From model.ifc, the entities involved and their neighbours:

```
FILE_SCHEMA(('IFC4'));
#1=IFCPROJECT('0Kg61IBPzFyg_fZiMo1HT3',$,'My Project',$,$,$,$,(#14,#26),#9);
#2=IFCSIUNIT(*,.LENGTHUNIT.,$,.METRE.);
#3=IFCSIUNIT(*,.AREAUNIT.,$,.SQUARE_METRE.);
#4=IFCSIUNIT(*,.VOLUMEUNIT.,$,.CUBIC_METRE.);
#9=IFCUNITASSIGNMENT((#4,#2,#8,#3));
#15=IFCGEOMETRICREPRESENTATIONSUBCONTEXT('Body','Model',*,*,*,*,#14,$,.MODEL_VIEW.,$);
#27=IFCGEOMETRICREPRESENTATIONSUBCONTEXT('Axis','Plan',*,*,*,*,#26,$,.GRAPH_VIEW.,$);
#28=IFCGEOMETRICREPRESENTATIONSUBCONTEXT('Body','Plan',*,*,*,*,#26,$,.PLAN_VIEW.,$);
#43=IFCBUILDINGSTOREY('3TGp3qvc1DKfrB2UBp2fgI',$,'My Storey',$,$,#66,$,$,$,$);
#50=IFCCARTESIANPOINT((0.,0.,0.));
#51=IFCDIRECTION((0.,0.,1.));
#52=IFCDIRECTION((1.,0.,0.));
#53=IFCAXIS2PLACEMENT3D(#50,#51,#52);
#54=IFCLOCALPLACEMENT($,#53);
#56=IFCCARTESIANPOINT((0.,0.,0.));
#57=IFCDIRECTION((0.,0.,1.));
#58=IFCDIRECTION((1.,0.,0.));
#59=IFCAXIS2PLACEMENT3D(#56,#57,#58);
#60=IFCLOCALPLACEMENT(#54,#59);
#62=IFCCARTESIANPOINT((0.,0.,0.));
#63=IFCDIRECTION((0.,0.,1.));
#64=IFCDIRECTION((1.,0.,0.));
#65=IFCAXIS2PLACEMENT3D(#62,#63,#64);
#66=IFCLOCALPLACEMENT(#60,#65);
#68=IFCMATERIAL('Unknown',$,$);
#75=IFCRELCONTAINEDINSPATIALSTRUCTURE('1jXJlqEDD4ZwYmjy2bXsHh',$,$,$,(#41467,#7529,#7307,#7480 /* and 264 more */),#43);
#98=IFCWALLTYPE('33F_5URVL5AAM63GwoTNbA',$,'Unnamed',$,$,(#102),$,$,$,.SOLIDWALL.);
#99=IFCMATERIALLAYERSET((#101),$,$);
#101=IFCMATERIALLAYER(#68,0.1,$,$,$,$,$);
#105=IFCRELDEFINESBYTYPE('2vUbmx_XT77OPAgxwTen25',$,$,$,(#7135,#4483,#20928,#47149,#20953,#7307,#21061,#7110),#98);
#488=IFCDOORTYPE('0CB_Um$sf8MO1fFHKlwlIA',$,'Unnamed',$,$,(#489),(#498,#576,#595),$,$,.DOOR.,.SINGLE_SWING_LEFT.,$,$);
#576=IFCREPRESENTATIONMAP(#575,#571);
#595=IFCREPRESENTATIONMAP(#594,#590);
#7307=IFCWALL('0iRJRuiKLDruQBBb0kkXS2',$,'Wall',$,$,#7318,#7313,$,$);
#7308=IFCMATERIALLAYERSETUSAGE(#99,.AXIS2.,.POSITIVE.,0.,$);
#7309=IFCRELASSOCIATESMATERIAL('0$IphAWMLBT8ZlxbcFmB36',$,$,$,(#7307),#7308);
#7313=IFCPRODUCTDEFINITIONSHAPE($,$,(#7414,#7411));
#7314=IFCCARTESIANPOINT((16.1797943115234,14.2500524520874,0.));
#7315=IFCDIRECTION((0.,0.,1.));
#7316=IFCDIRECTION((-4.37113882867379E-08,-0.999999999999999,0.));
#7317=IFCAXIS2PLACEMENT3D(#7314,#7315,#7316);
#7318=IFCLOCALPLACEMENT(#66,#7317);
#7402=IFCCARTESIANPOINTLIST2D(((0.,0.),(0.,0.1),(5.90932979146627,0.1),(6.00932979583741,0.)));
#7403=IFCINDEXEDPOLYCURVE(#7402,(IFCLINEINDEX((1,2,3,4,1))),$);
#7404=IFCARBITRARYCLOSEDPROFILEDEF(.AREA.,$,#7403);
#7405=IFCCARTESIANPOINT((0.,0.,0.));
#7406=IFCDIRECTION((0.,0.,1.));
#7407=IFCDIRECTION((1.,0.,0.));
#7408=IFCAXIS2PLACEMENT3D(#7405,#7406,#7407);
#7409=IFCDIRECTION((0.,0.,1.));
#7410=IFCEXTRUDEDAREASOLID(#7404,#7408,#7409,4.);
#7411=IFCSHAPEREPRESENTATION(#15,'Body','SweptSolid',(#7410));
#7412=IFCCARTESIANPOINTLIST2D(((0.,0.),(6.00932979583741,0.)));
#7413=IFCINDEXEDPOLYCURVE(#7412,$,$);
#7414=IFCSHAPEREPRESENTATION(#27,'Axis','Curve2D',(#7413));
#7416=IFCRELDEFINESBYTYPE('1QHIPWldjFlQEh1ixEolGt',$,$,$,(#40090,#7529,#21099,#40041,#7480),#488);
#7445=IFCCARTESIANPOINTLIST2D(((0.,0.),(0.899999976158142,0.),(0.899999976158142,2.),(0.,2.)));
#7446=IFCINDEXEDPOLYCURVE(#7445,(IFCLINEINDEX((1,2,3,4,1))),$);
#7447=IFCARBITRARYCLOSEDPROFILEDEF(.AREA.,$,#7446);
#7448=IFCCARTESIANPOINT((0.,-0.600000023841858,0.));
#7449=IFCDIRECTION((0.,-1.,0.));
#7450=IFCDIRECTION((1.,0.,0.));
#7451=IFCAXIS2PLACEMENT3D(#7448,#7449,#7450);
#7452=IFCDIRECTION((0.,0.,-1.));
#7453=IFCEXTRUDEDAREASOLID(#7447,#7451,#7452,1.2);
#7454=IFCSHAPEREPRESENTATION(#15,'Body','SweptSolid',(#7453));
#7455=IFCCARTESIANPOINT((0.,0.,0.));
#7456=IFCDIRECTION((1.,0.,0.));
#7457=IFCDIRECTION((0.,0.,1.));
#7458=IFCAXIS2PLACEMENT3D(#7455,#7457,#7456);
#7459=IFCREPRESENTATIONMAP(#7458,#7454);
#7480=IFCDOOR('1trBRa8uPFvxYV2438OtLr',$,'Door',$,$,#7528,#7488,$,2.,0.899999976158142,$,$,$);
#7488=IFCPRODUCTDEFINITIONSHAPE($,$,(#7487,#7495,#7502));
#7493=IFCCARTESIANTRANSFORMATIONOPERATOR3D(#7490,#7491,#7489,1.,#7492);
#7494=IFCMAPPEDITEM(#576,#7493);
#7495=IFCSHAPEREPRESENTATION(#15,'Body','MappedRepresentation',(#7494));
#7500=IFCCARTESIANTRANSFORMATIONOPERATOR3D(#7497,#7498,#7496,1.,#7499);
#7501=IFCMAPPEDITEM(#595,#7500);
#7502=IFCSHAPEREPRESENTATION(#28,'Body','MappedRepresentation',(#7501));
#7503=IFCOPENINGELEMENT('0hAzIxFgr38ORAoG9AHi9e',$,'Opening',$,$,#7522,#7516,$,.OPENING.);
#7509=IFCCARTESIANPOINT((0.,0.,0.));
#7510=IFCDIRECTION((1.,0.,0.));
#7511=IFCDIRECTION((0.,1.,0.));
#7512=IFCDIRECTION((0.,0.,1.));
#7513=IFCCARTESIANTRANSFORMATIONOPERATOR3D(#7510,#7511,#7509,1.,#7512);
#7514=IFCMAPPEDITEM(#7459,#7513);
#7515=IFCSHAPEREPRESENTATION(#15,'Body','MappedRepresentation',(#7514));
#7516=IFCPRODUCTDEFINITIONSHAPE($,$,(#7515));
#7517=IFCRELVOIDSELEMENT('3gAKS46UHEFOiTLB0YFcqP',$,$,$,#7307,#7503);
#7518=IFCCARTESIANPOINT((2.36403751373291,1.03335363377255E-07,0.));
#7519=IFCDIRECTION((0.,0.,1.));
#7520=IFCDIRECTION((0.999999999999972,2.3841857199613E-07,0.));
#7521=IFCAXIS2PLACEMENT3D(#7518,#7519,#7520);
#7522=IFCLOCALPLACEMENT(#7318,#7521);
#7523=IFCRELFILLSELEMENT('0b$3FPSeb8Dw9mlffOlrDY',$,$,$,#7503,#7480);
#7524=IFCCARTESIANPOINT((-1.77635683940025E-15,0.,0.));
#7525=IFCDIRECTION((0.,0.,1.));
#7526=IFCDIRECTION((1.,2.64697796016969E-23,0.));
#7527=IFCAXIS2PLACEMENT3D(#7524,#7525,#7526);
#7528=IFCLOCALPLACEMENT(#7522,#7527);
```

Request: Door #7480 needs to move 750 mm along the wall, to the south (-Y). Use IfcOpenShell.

```python
import ifcopenshell
import ifcopenshell.api.geometry
import ifcopenshell.util.placement

model = ifcopenshell.open("model.ifc")

door = model.by_guid("1trBRa8uPFvxYV2438OtLr")
opening = door.FillsVoids[0].RelatingOpeningElement
wall = opening.VoidsElements[0].RelatingBuildingElement

wall_matrix = ifcopenshell.util.placement.get_local_placement(wall.ObjectPlacement)
shift = wall_matrix[:3, 0] * 0.75
before = ifcopenshell.util.placement.get_local_placement(door.ObjectPlacement)[:3, 3].copy()

# The door is placed relative to its opening, so it follows when the opening moves.
matrix = ifcopenshell.util.placement.get_local_placement(opening.ObjectPlacement)
matrix[:3, 3] += shift
ifcopenshell.api.geometry.edit_object_placement(
    model, product=opening, matrix=matrix, is_si=False, should_transform_children=True
)

after = ifcopenshell.util.placement.get_local_placement(door.ObjectPlacement)[:3, 3]
print("door moved by", (after - before).round(3) + 0.0)

model.write("model_v2.ifc")
```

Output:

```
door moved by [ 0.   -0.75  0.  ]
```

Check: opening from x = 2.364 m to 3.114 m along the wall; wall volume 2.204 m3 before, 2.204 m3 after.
